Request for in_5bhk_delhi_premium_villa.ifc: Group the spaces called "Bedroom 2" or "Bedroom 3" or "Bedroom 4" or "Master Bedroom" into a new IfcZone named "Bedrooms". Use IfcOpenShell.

First a look at what the model holds.

```python
import ifcopenshell

model = ifcopenshell.open("in_5bhk_delhi_premium_villa.ifc")
print(model.schema)
seen = {}
for space in model.by_type("IfcSpace"):
    seen[space.LongName] = seen.get(space.LongName, 0) + 1
for name, count in sorted(seen.items(), key=str):
    print(count, "x", name)
print("zones:", [z.Name for z in model.by_type("IfcZone")][:20])
```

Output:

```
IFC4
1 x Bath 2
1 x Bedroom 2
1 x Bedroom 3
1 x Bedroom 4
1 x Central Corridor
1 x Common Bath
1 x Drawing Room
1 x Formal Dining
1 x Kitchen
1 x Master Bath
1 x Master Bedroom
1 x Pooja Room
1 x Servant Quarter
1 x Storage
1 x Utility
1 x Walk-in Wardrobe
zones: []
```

```python
import ifcopenshell
import ifcopenshell.api.group
import ifcopenshell.api.root

model = ifcopenshell.open("in_5bhk_delhi_premium_villa.ifc")

names = {"Bedroom 2", "Bedroom 3", "Bedroom 4", "Master Bedroom"}
spaces = [s for s in model.by_type("IfcSpace") if s.LongName in names]

zone = ifcopenshell.api.root.create_entity(model, ifc_class="IfcZone", name="Bedrooms")
ifcopenshell.api.group.assign_group(model, products=spaces, group=zone)
print(len(spaces), "spaces in", zone.Name)

model.write("in_5bhk_delhi_premium_villa_rev.ifc")
```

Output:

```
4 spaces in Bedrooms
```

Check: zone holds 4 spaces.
